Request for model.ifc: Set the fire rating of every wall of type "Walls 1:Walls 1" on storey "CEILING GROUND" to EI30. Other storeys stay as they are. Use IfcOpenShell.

First a look at what the model holds.

```python
import ifcopenshell
import ifcopenshell.util.element

model = ifcopenshell.open("model.ifc")
print(model.schema)
storey = next(s for s in model.by_type("IfcBuildingStorey") if s.Name == "CEILING GROUND")
walls = [e for e in ifcopenshell.util.element.get_decomposition(storey) if e.is_a("IfcWall")]
seen = {}
for e in walls:
    element_type = ifcopenshell.util.element.get_type(e)
    key = (element_type.Name if element_type != e and element_type else None, ifcopenshell.util.element.get_pset(e, "Pset_WallCommon", "FireRating"))
    seen[key] = seen.get(key, 0) + 1
for (name, value), count in sorted(seen.items(), key=str):
    print(count, "x", name, "|", value)
```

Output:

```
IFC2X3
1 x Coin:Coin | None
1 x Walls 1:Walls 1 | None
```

```python
import ifcopenshell
import ifcopenshell.api.pset
import ifcopenshell.util.element

model = ifcopenshell.open("model.ifc")

storey = next(s for s in model.by_type("IfcBuildingStorey") if s.Name == "CEILING GROUND")
walls = [e for e in ifcopenshell.util.element.get_decomposition(storey) if e.is_a("IfcWall")]

count = 0
for e in walls:
    element_type = ifcopenshell.util.element.get_type(e)
    if element_type in (None, e) or element_type.Name != "Walls 1:Walls 1":
        continue
    # add_pset returns the element's existing set when there is one.
    pset = ifcopenshell.api.pset.add_pset(model, product=e, name="Pset_WallCommon")
    ifcopenshell.api.pset.edit_pset(model, pset=pset, properties={"FireRating": "EI30"})
    count += 1

print(count, "walls updated")

model.write("model-out.ifc")
```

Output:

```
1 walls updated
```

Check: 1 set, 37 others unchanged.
